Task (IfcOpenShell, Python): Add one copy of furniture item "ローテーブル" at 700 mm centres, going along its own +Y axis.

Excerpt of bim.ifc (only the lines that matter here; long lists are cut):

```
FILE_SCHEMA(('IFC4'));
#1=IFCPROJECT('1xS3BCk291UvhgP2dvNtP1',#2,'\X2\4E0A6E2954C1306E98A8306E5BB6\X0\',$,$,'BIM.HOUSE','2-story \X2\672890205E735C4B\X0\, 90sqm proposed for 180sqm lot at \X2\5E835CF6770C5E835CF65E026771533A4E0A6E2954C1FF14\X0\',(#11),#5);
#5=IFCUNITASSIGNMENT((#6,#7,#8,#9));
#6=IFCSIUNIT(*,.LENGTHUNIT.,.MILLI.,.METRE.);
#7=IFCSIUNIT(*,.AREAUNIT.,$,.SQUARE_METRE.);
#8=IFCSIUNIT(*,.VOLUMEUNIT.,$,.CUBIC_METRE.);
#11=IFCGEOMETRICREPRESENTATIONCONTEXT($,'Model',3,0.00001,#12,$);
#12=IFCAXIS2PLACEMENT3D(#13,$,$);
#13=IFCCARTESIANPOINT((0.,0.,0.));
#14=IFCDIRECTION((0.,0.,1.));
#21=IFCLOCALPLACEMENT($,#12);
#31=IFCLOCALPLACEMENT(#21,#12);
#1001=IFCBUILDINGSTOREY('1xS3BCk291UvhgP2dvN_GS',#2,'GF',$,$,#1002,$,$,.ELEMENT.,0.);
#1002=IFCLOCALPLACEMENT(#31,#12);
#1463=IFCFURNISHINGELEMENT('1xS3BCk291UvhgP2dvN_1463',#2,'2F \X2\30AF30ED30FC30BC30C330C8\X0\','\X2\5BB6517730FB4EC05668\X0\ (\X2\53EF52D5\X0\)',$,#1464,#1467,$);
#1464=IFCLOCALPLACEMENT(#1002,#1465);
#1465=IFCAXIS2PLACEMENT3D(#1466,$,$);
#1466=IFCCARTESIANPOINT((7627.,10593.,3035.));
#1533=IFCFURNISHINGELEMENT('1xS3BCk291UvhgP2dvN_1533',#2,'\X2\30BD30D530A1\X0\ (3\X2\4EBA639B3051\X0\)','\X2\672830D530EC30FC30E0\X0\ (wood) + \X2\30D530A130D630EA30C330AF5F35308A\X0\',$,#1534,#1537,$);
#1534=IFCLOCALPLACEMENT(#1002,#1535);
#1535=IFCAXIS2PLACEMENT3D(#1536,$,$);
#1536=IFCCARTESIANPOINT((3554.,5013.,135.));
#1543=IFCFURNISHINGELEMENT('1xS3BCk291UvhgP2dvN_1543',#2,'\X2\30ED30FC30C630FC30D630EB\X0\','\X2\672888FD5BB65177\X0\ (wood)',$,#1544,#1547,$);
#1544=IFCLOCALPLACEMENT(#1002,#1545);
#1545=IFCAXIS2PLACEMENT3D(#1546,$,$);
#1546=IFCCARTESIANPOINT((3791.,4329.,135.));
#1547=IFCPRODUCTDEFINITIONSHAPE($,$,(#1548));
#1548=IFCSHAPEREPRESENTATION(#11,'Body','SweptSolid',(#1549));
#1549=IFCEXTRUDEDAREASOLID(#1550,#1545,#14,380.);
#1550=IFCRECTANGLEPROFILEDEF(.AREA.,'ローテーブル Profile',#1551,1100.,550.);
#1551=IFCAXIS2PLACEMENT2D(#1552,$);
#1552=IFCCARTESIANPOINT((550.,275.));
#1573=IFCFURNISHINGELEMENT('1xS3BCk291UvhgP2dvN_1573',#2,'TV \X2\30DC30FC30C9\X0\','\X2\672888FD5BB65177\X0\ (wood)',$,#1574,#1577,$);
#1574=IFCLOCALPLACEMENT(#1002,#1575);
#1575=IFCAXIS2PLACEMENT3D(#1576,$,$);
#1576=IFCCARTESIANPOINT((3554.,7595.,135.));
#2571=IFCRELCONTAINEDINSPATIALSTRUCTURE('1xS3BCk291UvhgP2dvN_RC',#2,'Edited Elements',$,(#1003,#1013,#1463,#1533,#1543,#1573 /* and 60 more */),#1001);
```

```python
import ifcopenshell
import ifcopenshell.api.geometry
import ifcopenshell.api.root
import ifcopenshell.util.element
import ifcopenshell.util.placement
import ifcopenshell.util.unit

model = ifcopenshell.open("bim.ifc")
unit_scale = ifcopenshell.util.unit.calculate_unit_scale(model)


def reuse_history(source, copy):
    """copy_class also copies each property set's owner history, people and application; keep the originals."""
    for rel in copy.IsDefinedBy:
        if rel.is_a("IfcRelDefinesByProperties") and (history := rel.RelatingPropertyDefinition.OwnerHistory):
            rel.RelatingPropertyDefinition.OwnerHistory = source.OwnerHistory
            ifcopenshell.util.element.remove_deep2(model, history)


source = model.by_id(1543)
base = ifcopenshell.util.placement.get_local_placement(source.ObjectPlacement)
step = base[:3, 1] * 0.7 / unit_scale

for i in range(1, 2):
    copy = ifcopenshell.api.root.copy_class(model, product=source)
    copy.Representation = ifcopenshell.util.element.copy_deep(
        model, source.Representation, exclude=["IfcGeometricRepresentationContext", "IfcRepresentationMap"]
    )
    reuse_history(source, copy)
    matrix = base.copy()
    matrix[:3, 3] += i * step
    print("added at", matrix[:3, 3].round(3) + 0.0)
    ifcopenshell.api.geometry.edit_object_placement(model, product=copy, matrix=matrix, is_si=False)

model.write("bim_v2.ifc")
```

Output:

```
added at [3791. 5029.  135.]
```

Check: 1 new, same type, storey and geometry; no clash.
